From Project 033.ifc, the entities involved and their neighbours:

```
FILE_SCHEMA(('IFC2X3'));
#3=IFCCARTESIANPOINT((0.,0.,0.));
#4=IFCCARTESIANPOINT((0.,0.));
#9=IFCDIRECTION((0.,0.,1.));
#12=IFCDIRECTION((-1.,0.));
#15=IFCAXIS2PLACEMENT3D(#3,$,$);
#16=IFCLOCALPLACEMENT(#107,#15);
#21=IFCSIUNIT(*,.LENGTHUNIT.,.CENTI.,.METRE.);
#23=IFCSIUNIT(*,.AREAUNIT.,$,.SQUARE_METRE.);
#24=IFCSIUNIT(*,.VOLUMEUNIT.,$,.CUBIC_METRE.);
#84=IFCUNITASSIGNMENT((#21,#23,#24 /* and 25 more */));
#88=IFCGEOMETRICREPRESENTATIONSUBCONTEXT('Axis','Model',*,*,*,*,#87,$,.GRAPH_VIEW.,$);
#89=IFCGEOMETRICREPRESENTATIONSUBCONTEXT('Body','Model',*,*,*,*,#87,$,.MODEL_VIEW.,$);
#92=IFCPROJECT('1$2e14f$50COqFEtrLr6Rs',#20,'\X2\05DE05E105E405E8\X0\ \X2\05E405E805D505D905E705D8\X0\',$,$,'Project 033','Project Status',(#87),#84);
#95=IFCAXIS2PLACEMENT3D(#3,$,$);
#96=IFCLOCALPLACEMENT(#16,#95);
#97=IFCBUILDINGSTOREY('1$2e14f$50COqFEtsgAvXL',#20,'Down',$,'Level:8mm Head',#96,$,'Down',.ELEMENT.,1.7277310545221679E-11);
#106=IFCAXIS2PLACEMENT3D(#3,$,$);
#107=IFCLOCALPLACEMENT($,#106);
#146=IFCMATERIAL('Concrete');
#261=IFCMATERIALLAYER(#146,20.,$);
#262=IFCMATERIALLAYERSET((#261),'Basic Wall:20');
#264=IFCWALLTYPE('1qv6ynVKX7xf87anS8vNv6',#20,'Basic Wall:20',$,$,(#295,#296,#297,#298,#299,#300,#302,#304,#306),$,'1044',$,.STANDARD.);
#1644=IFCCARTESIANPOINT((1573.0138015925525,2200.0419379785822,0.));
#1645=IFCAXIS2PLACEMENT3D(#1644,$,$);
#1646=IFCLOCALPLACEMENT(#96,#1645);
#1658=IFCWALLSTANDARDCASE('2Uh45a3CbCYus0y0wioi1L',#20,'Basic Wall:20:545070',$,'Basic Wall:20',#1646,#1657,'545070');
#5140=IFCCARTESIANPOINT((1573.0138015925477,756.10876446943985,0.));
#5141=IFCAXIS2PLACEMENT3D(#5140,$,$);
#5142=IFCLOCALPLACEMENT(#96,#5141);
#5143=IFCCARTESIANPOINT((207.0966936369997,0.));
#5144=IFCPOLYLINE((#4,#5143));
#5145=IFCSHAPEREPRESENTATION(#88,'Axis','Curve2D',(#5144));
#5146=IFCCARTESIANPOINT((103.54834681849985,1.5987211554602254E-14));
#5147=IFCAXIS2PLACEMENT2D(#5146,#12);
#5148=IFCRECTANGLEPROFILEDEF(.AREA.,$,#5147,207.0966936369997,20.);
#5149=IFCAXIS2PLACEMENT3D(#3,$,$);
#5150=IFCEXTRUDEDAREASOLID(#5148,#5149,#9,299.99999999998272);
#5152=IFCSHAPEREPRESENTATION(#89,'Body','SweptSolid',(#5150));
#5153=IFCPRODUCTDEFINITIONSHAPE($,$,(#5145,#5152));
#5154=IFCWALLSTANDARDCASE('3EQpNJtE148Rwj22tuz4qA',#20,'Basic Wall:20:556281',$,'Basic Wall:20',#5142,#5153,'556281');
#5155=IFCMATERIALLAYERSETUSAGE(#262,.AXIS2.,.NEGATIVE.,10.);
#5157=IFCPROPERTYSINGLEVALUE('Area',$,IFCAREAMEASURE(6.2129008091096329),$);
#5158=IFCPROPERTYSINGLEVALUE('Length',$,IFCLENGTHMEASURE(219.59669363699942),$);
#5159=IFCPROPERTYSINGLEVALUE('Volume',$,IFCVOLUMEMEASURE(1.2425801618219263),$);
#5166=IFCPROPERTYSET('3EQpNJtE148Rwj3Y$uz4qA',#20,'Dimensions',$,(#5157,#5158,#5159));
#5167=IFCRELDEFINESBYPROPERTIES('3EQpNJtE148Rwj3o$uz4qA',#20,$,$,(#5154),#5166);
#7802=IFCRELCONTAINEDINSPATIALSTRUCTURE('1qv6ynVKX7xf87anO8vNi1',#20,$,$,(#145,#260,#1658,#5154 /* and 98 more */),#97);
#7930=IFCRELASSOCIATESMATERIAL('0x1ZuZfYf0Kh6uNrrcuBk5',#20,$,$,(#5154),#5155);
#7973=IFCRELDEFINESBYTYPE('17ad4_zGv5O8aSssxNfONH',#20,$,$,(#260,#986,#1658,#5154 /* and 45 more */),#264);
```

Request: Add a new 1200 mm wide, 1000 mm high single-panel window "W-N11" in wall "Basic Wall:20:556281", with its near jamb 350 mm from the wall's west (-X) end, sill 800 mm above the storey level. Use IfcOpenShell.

```python
import numpy as np
import ifcopenshell
import ifcopenshell.api.feature
import ifcopenshell.api.geometry
import ifcopenshell.api.pset
import ifcopenshell.api.root
import ifcopenshell.api.spatial
import ifcopenshell.api.type
import ifcopenshell.geom
import ifcopenshell.util.element
import ifcopenshell.util.placement
import ifcopenshell.util.representation
import ifcopenshell.util.shape
import ifcopenshell.util.unit

model = ifcopenshell.open("Project 033.ifc")
unit_scale = ifcopenshell.util.unit.calculate_unit_scale(model)
area_scale = ifcopenshell.util.unit.calculate_unit_scale(model, "AREAUNIT")
volume_scale = ifcopenshell.util.unit.calculate_unit_scale(model, "VOLUMEUNIT")
settings = ifcopenshell.geom.settings()


def volume(element):
    """Net volume in cubic metres, openings subtracted."""
    shape = ifcopenshell.geom.create_shape(settings, element)
    return ifcopenshell.util.shape.get_volume(shape.geometry)


wall = model.by_guid("3EQpNJtE148Rwj22tuz4qA")
storey = ifcopenshell.util.element.get_container(wall, ifc_class="IfcBuildingStorey")
context = ifcopenshell.util.representation.get_context(model, "Model", "Body", "MODEL_VIEW")
before = volume(wall)

width, height, from_end, sill = 1.2, 1, 0.35, 0.8  # metres

# The wall runs along its own X axis, and the end named is its -X end.
wall_shape = ifcopenshell.geom.create_shape(settings, wall)
x, y, z = ifcopenshell.util.shape.get_vertices(wall_shape.geometry).T
start = x.min() + from_end
face, thickness = float(y.min()), float(y.max() - y.min())
wall_matrix = ifcopenshell.util.placement.get_local_placement(wall.ObjectPlacement)
level = ifcopenshell.util.placement.get_local_placement(storey.ObjectPlacement)[2, 3]


def in_wall(x, y):
    """Placement at x, y metres in the wall's axes, at sill height."""
    matrix = wall_matrix.copy()
    matrix[:, 3] = wall_matrix @ np.array([x / unit_scale, y / unit_scale, 0.0, 1.0])
    matrix[2, 3] = level + sill / unit_scale
    return matrix


# Opening: a box that overshoots both wall faces by 50 mm.
opening = ifcopenshell.api.root.create_entity(model, ifc_class="IfcOpeningElement")
box = ifcopenshell.api.geometry.add_wall_representation(
    model, context=context, length=width, height=height, thickness=thickness + 0.1
)
ifcopenshell.api.geometry.assign_representation(model, product=opening, representation=box)
ifcopenshell.api.geometry.edit_object_placement(model, product=opening, matrix=in_wall(start, face - 0.05), is_si=False)
ifcopenshell.api.feature.add_feature(model, feature=opening, element=wall)

window = ifcopenshell.api.root.create_entity(model, ifc_class="IfcWindow", name="W-N11")
window.OverallWidth, window.OverallHeight = width / unit_scale, height / unit_scale
body = ifcopenshell.api.geometry.add_window_representation(
    model,
    context=context,
    overall_width=window.OverallWidth,
    overall_height=window.OverallHeight,
    partition_type="SINGLE_PANEL",
)
ifcopenshell.api.geometry.assign_representation(model, product=window, representation=body)
ifcopenshell.api.spatial.assign_container(model, products=[window], relating_structure=storey)
fills = ifcopenshell.api.feature.add_filling(model, opening=opening, element=window)
fills.OwnerHistory = window.OwnerHistory  # required in IFC2X3

# IFC2X3 keeps the operation on the window style.
style = ifcopenshell.api.root.create_entity(model, ifc_class="IfcWindowStyle", name="W-N11")
style.OperationType, style.ConstructionType = "SINGLE_PANEL", "NOTDEFINED"
style.ParameterTakesPrecedence = style.Sizeable = False
ifcopenshell.api.type.assign_type(model, related_objects=[window], relating_type=style)

# Centre the window in the wall's thickness.
ifcopenshell.api.geometry.edit_object_placement(model, product=window, matrix=in_wall(start, face), is_si=False)
window_shape = ifcopenshell.geom.create_shape(settings, window)
depth = ifcopenshell.util.shape.get_vertices(window_shape.geometry)[:, 1]
offset = face + thickness / 2 - (depth.min() + depth.max()) / 2
ifcopenshell.api.geometry.edit_object_placement(model, product=window, matrix=in_wall(start, offset), is_si=False)

after = volume(wall)

# Update the wall's stored quantities.
pset = model.by_id(ifcopenshell.util.element.get_pset(wall, "Dimensions", should_inherit=False)["id"])
ifcopenshell.api.pset.edit_pset(model, pset=pset, properties={
    "Area": model.create_entity("IfcAreaMeasure", after / thickness / area_scale),
    "Volume": model.create_entity("IfcVolumeMeasure", after / volume_scale),
})

print(f"wall volume {before:.3f} -> {after:.3f} m3")

model.write("Project 033_rev.ifc")
```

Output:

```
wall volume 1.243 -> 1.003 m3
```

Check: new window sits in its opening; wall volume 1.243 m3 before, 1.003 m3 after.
